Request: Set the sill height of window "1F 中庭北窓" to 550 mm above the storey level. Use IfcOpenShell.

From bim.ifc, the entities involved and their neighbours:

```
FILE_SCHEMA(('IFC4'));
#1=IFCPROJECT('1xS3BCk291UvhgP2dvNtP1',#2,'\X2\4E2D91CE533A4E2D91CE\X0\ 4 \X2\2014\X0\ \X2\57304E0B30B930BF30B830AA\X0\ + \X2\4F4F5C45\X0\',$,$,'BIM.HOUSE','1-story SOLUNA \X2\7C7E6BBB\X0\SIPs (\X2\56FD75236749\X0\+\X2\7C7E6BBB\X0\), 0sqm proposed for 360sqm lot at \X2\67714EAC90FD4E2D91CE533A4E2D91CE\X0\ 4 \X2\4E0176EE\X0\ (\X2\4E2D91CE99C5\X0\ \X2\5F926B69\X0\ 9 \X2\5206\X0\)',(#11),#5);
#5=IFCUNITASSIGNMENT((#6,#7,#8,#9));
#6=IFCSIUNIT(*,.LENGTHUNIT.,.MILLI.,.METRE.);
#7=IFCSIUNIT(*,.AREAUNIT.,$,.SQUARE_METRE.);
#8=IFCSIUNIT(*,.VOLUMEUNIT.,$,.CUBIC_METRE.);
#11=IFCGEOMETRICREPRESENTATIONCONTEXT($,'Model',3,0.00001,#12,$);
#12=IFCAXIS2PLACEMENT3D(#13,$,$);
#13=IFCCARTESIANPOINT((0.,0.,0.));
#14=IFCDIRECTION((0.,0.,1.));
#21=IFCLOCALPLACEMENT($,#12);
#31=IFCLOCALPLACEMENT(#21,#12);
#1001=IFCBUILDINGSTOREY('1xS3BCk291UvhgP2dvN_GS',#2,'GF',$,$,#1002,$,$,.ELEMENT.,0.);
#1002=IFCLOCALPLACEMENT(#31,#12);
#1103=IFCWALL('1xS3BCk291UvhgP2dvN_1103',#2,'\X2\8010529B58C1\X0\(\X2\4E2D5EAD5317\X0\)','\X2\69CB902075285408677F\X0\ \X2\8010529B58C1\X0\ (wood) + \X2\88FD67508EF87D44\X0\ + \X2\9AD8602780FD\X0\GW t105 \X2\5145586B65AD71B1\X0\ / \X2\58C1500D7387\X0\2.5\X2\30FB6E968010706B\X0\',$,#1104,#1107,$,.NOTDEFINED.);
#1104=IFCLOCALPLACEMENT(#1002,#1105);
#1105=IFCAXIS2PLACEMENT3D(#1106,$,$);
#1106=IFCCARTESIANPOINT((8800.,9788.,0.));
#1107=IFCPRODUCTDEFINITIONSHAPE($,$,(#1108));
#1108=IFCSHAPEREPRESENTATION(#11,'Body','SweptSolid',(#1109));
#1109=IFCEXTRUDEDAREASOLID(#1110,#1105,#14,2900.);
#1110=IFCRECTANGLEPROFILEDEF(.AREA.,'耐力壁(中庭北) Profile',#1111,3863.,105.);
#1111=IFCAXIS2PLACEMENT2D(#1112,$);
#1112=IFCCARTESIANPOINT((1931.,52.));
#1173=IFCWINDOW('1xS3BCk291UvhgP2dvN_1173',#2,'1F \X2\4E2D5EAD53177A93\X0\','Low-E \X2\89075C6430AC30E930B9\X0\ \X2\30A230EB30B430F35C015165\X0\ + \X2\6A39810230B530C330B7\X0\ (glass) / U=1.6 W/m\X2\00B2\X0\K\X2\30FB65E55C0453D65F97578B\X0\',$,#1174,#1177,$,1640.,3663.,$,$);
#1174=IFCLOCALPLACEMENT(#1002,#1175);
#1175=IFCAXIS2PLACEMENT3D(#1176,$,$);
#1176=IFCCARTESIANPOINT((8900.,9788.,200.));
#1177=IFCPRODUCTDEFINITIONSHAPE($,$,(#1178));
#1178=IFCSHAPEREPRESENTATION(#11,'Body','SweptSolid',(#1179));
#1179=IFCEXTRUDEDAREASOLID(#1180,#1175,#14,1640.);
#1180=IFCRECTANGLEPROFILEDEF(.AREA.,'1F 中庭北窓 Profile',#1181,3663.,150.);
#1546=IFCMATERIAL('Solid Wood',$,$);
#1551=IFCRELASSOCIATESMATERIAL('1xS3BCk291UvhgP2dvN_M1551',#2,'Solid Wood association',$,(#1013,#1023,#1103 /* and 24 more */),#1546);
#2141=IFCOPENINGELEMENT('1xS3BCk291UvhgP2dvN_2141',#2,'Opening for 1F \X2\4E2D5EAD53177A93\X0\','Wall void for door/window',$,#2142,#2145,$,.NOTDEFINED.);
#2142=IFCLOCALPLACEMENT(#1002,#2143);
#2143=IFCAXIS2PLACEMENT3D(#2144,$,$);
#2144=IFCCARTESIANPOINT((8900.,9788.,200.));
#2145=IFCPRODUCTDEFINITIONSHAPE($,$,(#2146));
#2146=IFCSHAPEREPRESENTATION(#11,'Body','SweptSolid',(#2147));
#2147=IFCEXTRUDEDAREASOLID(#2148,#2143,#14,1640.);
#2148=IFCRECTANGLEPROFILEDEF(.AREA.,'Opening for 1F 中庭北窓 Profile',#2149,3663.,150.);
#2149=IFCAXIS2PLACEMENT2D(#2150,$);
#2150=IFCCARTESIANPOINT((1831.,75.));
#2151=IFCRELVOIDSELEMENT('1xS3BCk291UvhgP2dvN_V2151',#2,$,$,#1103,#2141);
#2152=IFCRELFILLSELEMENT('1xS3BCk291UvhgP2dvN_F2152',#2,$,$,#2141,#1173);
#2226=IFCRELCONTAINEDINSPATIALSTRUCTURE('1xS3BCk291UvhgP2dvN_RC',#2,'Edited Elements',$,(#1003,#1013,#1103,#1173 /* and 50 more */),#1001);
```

```python
import numpy as np
import ifcopenshell
import ifcopenshell.api.geometry
import ifcopenshell.geom
import ifcopenshell.util.element
import ifcopenshell.util.placement
import ifcopenshell.util.shape
import ifcopenshell.util.unit

model = ifcopenshell.open("bim.ifc")
unit_scale = ifcopenshell.util.unit.calculate_unit_scale(model)

window = model.by_guid("1xS3BCk291UvhgP2dvN_1173")
opening = window.FillsVoids[0].RelatingOpeningElement
storey = ifcopenshell.util.element.get_container(window, ifc_class="IfcBuildingStorey")
level = ifcopenshell.util.placement.get_local_placement(storey.ObjectPlacement)[2, 3]

# The opening's origin need not be at the sill, so measure its lowest point.
shape = ifcopenshell.geom.create_shape(ifcopenshell.geom.settings(), opening)
bottom = ifcopenshell.util.shape.get_shape_bottom_elevation(shape, shape.geometry) / unit_scale
dz = level + 550.0 - bottom

shift = np.array([0.0, 0.0, dz])
# The window is not placed relative to its opening, so move both.
for product in (opening, window):
    matrix = ifcopenshell.util.placement.get_local_placement(product.ObjectPlacement)
    matrix[:3, 3] += shift
    ifcopenshell.api.geometry.edit_object_placement(model, product=product, matrix=matrix, is_si=False)

print(f"moved by {dz * unit_scale:+.3f} m")

model.write("bim_rev.ifc")
```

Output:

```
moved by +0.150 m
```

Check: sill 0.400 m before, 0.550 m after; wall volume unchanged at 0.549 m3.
